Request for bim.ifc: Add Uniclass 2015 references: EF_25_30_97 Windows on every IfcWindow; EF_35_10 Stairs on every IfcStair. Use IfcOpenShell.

First a look at what the model holds.

```python
import ifcopenshell

model = ifcopenshell.open("bim.ifc")
print(model.schema)
print("classifications:", [c.Name for c in model.by_type("IfcClassification")])
for ifc_class in ("IfcDoor", "IfcRoof", "IfcStair", "IfcWall", "IfcWindow"):
    print(ifc_class, len(model.by_type(ifc_class)))
```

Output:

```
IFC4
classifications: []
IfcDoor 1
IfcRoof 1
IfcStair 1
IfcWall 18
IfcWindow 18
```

```python
import ifcopenshell
import ifcopenshell.api.classification

model = ifcopenshell.open("bim.ifc")

system = ifcopenshell.api.classification.add_classification(model, classification="Uniclass 2015")

codes = {
    "IfcWindow": ("EF_25_30_97", "Windows"),
    "IfcStair": ("EF_35_10", "Stairs"),
}
for ifc_class, (code, name) in codes.items():
    products = model.by_type(ifc_class)
    ifcopenshell.api.classification.add_reference(
        model, products=products, classification=system, identification=code, name=name
    )
    print(code, len(products))

model.write("bim_edited.ifc")
```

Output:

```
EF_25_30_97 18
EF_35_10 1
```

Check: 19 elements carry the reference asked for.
